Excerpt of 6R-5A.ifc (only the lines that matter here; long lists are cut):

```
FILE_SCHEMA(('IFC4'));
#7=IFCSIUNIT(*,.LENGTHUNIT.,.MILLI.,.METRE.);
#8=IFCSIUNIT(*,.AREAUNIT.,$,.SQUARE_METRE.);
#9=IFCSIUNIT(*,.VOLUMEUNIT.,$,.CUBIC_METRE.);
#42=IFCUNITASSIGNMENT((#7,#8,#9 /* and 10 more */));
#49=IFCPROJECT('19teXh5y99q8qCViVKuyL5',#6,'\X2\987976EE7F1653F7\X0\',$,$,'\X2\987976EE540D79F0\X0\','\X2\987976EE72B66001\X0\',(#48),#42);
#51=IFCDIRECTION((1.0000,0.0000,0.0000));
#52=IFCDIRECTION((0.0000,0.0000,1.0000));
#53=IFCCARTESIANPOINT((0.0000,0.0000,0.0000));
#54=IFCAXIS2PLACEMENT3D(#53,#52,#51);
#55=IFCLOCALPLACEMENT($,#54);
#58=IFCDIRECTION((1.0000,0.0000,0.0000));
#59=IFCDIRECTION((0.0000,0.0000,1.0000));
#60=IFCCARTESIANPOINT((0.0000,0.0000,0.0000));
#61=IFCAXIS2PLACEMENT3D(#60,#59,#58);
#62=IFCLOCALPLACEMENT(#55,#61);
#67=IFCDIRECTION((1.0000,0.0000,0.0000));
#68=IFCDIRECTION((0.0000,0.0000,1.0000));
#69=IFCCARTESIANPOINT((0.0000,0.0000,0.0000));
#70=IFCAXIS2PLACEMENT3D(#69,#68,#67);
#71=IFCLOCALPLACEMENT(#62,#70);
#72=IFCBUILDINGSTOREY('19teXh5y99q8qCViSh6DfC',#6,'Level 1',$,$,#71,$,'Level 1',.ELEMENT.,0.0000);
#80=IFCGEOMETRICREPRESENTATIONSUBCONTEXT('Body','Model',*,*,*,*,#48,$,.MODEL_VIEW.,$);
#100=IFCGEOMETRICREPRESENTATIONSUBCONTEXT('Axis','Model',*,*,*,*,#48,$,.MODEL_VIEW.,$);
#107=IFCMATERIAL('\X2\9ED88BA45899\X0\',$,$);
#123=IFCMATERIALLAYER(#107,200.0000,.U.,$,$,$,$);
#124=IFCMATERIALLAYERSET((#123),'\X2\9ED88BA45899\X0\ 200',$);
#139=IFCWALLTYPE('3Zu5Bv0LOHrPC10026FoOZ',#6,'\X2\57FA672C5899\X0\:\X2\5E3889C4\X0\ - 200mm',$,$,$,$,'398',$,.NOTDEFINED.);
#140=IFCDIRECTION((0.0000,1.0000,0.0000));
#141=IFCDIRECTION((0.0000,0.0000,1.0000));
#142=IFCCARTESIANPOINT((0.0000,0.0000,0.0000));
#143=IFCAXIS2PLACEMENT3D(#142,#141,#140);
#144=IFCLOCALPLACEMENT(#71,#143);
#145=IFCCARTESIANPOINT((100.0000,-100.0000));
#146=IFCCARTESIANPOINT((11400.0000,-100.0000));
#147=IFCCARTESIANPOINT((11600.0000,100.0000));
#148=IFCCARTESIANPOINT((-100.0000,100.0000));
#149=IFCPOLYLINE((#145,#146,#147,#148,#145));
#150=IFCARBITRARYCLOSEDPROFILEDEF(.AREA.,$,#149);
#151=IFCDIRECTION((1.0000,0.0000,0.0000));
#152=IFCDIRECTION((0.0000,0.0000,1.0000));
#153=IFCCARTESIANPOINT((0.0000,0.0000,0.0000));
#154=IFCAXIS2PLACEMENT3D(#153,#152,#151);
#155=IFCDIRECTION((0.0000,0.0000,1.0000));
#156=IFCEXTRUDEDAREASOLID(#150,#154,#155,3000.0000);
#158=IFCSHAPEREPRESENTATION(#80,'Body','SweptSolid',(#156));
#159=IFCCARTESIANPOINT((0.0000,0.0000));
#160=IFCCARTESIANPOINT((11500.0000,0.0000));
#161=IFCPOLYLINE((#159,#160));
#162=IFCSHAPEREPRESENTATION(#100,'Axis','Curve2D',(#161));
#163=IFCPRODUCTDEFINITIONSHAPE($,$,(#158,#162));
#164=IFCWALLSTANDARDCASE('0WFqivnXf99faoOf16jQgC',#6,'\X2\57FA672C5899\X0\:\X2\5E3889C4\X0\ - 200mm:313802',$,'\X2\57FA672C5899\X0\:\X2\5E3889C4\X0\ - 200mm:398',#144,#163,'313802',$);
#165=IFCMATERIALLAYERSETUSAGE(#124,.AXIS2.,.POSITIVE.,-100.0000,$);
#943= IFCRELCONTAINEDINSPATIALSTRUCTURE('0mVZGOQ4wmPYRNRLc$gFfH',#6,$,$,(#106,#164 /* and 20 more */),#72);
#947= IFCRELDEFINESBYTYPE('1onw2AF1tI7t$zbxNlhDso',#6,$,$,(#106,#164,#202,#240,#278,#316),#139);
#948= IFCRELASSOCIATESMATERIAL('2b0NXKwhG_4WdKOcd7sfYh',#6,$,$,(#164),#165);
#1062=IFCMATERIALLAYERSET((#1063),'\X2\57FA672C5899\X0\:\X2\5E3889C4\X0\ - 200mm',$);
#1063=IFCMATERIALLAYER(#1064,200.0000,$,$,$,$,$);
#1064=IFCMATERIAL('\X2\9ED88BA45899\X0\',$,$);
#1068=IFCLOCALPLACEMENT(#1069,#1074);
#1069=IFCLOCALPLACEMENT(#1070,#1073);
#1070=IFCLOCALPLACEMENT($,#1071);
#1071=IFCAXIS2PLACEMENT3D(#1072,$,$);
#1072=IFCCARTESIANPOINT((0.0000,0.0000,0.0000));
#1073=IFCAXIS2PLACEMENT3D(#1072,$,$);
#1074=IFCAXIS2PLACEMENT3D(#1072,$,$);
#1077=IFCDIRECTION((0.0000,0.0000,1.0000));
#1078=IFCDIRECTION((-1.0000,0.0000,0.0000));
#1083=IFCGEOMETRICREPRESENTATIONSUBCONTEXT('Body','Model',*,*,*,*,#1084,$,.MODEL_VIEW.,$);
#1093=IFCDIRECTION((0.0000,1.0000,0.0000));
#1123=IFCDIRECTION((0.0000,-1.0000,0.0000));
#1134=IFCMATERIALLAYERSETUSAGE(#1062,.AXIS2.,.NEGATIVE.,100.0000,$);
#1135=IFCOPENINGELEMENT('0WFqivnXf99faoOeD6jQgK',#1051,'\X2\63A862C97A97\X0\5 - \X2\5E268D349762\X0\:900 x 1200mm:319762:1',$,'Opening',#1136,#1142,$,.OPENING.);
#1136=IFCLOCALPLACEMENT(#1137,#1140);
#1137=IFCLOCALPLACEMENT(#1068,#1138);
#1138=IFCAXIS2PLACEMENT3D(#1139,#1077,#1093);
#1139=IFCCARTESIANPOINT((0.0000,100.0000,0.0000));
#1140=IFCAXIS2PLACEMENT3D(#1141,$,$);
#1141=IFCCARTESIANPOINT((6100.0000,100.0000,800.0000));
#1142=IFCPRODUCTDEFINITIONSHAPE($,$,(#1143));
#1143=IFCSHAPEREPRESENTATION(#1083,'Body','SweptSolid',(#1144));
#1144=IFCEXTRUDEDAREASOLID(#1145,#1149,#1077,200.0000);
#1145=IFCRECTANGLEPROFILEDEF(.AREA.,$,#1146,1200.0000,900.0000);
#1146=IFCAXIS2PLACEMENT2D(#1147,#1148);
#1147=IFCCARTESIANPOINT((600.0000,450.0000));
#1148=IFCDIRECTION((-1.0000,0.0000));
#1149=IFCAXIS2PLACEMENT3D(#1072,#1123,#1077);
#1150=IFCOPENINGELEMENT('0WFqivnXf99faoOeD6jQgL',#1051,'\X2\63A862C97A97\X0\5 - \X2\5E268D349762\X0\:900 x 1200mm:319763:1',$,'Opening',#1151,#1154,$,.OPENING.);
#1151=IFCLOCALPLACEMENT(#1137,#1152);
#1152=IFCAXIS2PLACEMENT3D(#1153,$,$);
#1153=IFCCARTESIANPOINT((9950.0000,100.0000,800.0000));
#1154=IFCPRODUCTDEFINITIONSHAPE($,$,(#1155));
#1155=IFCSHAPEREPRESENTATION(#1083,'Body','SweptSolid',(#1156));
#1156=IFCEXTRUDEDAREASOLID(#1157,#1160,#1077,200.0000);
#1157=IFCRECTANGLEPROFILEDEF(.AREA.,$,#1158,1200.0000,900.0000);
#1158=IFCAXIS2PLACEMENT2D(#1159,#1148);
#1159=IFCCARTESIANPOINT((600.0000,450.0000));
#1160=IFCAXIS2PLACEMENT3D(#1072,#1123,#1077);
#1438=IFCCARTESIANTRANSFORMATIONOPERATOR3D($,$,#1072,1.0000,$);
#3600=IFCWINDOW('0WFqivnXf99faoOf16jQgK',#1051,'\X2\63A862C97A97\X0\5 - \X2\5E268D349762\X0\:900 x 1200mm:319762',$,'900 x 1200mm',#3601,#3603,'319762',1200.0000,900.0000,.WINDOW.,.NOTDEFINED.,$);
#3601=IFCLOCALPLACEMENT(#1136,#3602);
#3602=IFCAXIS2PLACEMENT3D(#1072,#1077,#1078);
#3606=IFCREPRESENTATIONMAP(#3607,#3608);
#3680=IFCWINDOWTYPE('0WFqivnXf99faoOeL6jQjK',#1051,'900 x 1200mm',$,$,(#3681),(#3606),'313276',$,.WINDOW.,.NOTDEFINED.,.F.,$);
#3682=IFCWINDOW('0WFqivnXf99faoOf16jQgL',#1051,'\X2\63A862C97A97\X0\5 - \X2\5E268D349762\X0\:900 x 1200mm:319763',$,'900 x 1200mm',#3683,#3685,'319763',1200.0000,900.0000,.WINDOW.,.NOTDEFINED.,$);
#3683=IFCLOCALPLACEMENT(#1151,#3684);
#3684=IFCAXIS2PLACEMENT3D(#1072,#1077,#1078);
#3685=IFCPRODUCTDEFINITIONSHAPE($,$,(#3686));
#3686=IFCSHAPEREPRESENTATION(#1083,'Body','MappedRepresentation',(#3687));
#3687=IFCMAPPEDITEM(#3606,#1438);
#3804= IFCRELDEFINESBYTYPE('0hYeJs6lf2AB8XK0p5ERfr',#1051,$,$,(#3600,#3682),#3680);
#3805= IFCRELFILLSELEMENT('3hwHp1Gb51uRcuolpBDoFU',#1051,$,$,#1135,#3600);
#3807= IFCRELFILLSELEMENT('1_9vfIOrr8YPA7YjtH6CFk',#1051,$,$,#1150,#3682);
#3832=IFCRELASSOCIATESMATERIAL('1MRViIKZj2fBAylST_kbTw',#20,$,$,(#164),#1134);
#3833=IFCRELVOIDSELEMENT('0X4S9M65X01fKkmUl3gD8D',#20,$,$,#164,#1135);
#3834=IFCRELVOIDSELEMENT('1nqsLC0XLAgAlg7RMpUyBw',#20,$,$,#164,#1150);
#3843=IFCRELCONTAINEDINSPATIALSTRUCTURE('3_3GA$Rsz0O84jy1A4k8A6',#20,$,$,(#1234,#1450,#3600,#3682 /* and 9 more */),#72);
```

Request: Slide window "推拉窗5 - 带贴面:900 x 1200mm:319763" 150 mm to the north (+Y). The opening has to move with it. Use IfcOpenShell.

```python
import ifcopenshell
import ifcopenshell.api.geometry
import ifcopenshell.util.placement
import ifcopenshell.util.unit

model = ifcopenshell.open("6R-5A.ifc")
unit_scale = ifcopenshell.util.unit.calculate_unit_scale(model)

window = model.by_id(3682)
opening = window.FillsVoids[0].RelatingOpeningElement
wall = opening.VoidsElements[0].RelatingBuildingElement

wall_matrix = ifcopenshell.util.placement.get_local_placement(wall.ObjectPlacement)
shift = wall_matrix[:3, 0] * 0.15 / unit_scale
before = ifcopenshell.util.placement.get_local_placement(window.ObjectPlacement)[:3, 3].copy()

# The window is placed relative to its opening, so it follows when the opening moves.
matrix = ifcopenshell.util.placement.get_local_placement(opening.ObjectPlacement)
matrix[:3, 3] += shift
ifcopenshell.api.geometry.edit_object_placement(
    model, product=opening, matrix=matrix, is_si=False, should_transform_children=True
)

after = ifcopenshell.util.placement.get_local_placement(window.ObjectPlacement)[:3, 3]
print("window moved by", (after - before).round(3) + 0.0)

model.write("6R-5A_rev.ifc")
```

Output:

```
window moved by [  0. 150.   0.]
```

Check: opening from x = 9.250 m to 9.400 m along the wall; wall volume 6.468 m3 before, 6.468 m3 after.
